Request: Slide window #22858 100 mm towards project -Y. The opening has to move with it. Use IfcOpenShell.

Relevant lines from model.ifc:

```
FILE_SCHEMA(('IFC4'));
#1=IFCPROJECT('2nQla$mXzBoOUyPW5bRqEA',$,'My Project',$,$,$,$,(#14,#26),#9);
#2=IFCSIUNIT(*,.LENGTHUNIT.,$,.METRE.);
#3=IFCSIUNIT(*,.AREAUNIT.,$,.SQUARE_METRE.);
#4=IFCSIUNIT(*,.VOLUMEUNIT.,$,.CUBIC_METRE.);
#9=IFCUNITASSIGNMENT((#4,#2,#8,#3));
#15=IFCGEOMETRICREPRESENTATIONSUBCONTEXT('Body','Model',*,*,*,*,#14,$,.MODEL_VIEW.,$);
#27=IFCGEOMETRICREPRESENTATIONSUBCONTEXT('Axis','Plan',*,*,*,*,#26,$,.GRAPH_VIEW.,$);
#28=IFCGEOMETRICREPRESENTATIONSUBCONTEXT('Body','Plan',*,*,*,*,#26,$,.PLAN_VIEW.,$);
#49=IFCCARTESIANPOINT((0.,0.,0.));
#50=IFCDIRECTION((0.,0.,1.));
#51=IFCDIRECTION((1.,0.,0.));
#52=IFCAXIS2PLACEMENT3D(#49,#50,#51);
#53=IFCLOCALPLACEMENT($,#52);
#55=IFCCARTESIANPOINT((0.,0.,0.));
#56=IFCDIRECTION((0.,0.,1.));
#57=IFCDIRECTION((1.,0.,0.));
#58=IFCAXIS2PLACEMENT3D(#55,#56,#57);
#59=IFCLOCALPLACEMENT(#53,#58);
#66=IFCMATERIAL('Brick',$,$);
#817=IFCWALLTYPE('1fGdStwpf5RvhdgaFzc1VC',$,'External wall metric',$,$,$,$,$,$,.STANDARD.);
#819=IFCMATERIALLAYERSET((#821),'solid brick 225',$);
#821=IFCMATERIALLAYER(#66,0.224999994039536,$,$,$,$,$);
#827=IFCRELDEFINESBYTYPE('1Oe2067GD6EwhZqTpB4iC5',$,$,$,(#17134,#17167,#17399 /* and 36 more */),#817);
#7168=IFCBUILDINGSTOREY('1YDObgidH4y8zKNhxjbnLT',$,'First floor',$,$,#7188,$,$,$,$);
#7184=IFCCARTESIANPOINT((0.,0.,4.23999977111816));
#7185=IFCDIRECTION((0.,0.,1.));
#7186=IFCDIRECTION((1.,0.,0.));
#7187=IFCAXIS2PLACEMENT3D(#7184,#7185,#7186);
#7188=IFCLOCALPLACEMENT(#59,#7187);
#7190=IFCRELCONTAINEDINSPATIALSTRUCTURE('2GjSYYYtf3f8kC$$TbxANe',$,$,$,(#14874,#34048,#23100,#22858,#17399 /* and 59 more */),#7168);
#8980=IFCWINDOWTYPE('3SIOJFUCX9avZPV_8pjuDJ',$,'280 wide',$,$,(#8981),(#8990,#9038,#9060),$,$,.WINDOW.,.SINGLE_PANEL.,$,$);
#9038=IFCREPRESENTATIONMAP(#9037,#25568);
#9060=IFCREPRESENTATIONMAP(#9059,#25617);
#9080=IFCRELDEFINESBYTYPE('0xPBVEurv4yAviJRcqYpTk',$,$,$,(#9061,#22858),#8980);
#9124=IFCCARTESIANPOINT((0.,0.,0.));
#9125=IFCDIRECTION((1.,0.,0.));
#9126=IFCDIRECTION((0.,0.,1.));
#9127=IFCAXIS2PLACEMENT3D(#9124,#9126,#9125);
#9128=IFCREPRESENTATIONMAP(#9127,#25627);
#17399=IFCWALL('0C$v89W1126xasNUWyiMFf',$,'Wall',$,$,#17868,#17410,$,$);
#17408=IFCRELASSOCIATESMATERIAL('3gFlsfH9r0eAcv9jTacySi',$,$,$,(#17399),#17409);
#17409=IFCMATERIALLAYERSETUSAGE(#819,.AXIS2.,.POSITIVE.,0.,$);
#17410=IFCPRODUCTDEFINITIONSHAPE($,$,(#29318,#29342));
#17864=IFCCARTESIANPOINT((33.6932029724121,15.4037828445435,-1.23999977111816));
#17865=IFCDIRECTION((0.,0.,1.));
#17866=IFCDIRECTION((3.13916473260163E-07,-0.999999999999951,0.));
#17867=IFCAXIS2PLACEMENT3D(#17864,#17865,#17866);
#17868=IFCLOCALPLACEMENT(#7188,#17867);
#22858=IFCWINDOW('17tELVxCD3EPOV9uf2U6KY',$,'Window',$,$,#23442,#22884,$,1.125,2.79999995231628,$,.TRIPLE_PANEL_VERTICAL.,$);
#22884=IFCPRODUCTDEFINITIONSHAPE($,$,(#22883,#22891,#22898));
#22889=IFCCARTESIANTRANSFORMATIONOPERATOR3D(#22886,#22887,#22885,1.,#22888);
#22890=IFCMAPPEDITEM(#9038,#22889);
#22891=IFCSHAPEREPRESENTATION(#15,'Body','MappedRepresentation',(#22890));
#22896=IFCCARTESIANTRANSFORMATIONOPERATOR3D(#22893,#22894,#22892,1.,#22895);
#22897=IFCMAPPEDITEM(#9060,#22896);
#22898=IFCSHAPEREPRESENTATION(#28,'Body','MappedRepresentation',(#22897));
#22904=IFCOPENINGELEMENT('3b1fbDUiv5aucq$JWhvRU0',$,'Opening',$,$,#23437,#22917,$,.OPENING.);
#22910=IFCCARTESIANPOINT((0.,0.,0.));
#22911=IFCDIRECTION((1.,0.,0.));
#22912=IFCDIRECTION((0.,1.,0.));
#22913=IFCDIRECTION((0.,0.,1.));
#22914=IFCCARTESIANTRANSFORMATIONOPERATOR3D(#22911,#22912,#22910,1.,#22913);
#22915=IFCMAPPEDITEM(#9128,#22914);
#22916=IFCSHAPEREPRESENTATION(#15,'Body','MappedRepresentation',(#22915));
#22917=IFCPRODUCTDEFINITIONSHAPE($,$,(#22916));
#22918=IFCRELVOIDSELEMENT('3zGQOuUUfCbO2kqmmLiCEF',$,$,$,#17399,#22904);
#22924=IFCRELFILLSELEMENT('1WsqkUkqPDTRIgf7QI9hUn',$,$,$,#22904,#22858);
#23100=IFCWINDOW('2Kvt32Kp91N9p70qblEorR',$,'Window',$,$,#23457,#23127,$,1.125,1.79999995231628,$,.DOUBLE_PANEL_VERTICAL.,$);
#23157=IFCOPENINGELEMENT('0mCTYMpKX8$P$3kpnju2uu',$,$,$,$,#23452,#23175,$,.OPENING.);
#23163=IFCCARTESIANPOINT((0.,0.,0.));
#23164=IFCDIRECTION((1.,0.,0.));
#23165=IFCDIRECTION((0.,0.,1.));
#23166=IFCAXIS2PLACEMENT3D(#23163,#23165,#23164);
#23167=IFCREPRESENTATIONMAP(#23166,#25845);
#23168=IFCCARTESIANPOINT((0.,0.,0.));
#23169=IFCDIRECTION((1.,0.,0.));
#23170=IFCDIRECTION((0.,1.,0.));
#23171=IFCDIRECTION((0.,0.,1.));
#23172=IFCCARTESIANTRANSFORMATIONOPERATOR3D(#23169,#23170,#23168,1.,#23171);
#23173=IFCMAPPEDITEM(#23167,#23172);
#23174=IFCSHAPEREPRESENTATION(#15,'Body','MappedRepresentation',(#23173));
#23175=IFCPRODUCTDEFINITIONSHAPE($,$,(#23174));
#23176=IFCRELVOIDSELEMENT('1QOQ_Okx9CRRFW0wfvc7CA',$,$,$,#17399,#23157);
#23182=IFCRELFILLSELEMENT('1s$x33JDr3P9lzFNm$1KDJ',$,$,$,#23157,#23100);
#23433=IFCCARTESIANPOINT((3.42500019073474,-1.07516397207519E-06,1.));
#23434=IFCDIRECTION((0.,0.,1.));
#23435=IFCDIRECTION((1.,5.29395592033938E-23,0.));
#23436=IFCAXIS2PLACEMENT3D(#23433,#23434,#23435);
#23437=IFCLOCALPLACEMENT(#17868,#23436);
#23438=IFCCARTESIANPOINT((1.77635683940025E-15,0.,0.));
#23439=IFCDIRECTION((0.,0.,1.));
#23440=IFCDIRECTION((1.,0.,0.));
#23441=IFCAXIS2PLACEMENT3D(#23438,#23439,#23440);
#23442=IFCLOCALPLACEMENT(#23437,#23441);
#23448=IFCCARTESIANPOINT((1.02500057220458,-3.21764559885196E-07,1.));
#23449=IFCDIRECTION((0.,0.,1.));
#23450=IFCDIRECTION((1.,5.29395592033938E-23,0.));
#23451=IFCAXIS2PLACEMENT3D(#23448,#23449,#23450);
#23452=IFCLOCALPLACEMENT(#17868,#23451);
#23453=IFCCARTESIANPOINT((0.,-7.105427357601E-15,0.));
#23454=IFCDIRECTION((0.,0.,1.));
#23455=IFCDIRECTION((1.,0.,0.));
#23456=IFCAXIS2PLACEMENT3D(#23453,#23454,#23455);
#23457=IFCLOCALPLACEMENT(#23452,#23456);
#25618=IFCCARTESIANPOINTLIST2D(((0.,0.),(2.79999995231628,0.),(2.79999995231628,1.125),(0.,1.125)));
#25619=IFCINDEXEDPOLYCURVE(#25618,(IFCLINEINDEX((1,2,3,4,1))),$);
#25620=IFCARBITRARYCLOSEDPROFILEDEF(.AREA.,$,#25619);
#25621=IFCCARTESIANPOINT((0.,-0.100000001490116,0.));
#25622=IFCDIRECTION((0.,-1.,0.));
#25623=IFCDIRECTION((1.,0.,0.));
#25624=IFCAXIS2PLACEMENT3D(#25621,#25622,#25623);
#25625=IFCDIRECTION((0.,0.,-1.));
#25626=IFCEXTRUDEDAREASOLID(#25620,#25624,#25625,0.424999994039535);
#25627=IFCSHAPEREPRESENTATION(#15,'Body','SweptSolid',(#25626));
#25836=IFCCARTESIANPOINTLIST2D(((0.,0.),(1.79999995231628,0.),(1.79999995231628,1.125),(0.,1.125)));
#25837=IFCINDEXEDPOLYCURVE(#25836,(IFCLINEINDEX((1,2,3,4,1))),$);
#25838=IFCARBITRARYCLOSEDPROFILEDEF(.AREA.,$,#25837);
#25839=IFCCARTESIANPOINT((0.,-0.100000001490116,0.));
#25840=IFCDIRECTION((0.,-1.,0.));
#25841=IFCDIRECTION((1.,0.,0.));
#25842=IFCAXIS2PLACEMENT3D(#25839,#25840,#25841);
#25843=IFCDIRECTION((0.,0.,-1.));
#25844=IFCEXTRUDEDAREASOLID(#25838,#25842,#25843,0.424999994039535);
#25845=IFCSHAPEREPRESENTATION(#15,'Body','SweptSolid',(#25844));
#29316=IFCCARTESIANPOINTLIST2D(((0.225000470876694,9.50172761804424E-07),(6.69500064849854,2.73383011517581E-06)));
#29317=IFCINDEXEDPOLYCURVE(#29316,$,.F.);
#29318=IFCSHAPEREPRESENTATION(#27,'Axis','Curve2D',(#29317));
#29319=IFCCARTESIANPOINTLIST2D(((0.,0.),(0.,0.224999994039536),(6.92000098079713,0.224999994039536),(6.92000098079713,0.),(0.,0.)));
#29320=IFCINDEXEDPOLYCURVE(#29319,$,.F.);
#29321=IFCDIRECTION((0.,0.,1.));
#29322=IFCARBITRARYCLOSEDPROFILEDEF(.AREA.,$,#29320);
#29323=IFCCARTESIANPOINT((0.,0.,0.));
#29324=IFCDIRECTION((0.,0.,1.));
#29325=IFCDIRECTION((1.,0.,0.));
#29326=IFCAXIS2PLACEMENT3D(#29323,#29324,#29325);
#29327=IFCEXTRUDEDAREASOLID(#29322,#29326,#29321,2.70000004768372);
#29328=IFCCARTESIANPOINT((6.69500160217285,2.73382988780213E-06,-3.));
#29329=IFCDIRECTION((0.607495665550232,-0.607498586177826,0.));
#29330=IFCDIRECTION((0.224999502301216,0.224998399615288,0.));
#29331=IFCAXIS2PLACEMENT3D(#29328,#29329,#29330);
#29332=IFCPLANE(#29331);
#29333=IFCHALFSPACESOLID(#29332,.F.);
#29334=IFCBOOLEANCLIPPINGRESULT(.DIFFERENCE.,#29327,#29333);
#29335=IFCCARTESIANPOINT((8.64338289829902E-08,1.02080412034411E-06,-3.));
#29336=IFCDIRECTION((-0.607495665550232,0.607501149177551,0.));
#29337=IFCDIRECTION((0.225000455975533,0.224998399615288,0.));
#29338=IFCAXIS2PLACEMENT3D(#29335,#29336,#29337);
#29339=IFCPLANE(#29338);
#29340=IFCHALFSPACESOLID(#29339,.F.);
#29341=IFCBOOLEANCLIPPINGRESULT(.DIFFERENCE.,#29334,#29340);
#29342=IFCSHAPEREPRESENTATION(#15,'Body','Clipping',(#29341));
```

```python
import ifcopenshell
import ifcopenshell.api.geometry
import ifcopenshell.util.placement
import ifcopenshell.util.unit

model = ifcopenshell.open("model.ifc")
unit_scale = ifcopenshell.util.unit.calculate_unit_scale(model)

window = model.by_guid("17tELVxCD3EPOV9uf2U6KY")
opening = window.FillsVoids[0].RelatingOpeningElement
wall = opening.VoidsElements[0].RelatingBuildingElement

wall_matrix = ifcopenshell.util.placement.get_local_placement(wall.ObjectPlacement)
shift = wall_matrix[:3, 0] * 0.1 / unit_scale
before = ifcopenshell.util.placement.get_local_placement(window.ObjectPlacement)[:3, 3].copy()

# The window is placed relative to its opening, so it follows when the opening moves.
matrix = ifcopenshell.util.placement.get_local_placement(opening.ObjectPlacement)
matrix[:3, 3] += shift
ifcopenshell.api.geometry.edit_object_placement(
    model, product=opening, matrix=matrix, is_si=False, should_transform_children=True
)

after = ifcopenshell.util.placement.get_local_placement(window.ObjectPlacement)[:3, 3]
print("window moved by", (after - before).round(3) + 0.0)

model.write("model_updated.ifc")
```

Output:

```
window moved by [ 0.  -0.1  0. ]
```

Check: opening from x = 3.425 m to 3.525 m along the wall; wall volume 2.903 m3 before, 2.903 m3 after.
